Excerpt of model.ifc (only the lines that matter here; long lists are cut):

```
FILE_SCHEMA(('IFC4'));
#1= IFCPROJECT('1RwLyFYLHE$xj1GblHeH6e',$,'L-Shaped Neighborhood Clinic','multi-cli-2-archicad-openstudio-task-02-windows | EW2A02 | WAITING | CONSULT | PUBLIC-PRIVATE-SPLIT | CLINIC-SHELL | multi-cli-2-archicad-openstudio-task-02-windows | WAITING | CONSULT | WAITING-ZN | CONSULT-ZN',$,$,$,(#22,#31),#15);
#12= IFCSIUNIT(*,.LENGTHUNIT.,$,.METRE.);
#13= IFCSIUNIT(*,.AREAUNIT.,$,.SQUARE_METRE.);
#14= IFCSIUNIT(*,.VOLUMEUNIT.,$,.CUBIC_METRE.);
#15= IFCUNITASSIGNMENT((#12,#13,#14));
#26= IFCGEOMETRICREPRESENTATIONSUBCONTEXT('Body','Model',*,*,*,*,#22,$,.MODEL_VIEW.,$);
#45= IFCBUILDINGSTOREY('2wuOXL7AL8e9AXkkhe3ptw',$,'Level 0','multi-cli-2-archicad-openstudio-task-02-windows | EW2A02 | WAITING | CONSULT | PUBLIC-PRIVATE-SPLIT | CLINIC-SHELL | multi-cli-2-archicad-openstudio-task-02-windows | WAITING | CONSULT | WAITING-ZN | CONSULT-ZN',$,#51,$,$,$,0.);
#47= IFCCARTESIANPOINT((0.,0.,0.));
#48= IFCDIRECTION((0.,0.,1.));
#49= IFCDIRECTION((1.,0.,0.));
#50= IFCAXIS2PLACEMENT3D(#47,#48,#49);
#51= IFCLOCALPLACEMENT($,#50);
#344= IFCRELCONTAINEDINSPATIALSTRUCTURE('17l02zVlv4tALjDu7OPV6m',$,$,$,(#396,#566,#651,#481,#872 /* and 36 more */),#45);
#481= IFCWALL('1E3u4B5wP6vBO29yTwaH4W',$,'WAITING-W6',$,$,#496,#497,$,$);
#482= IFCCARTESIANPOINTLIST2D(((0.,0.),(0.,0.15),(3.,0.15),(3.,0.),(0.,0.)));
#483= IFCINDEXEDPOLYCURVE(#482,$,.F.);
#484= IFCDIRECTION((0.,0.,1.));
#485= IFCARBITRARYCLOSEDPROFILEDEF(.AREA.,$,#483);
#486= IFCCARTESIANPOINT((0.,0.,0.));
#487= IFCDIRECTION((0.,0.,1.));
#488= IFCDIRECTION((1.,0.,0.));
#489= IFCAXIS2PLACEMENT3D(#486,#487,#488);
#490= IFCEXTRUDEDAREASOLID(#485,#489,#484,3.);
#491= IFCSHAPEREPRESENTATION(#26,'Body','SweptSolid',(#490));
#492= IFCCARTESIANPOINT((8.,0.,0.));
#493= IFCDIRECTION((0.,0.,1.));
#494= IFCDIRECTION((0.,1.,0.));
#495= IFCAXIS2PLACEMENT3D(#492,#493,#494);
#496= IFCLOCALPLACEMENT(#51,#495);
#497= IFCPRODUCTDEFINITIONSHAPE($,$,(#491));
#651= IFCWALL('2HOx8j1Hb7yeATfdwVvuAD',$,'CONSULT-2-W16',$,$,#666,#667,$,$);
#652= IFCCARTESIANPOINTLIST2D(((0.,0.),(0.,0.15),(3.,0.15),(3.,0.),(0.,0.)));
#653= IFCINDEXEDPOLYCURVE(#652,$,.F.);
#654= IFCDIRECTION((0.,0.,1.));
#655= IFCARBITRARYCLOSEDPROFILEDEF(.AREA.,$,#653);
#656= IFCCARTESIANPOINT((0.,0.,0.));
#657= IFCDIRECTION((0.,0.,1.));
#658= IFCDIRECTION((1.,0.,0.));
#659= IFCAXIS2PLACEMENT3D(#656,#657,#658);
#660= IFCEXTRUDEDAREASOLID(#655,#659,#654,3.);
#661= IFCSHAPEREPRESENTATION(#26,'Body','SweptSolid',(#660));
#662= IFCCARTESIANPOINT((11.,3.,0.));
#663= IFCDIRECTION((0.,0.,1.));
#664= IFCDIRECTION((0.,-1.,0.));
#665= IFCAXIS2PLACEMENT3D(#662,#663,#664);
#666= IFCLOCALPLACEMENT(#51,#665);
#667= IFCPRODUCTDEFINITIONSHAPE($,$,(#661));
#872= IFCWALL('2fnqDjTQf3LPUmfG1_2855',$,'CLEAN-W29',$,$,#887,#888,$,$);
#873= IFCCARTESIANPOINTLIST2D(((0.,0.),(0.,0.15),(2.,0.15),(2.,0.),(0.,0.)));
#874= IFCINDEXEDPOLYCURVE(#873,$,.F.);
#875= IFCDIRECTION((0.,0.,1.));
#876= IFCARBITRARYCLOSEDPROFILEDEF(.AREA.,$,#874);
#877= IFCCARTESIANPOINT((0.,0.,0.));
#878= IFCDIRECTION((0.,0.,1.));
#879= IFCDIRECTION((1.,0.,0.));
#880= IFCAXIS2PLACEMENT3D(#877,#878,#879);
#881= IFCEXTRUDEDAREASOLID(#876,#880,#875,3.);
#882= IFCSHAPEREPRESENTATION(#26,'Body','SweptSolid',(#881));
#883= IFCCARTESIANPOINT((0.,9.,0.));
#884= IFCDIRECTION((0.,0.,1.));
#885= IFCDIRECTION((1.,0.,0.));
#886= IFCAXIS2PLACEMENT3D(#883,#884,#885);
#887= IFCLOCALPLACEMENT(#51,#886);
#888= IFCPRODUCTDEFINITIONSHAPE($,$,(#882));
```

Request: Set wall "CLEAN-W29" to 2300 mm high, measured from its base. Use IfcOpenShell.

```python
import ifcopenshell
import ifcopenshell.geom
import ifcopenshell.util.representation
import ifcopenshell.util.shape
import ifcopenshell.util.unit

model = ifcopenshell.open("model.ifc")
unit_scale = ifcopenshell.util.unit.calculate_unit_scale(model)
settings = ifcopenshell.geom.settings()


def volume(element):
    """Net volume in cubic metres, openings subtracted."""
    shape = ifcopenshell.geom.create_shape(settings, element)
    return ifcopenshell.util.shape.get_volume(shape.geometry)


wall = model.by_id(872)
before = volume(wall)

body = ifcopenshell.util.representation.get_representation(wall, "Model", "Body")
solid = body.Items[0]
old_height = solid.Depth
solid.Depth = 2.3 / unit_scale
after = volume(wall)

print(f"height {old_height:g} -> {solid.Depth:g}, volume {before:.3f} -> {after:.3f} m3")

model.write("model_edited.ifc")
```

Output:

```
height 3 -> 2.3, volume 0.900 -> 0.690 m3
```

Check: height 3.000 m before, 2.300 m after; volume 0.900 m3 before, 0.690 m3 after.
